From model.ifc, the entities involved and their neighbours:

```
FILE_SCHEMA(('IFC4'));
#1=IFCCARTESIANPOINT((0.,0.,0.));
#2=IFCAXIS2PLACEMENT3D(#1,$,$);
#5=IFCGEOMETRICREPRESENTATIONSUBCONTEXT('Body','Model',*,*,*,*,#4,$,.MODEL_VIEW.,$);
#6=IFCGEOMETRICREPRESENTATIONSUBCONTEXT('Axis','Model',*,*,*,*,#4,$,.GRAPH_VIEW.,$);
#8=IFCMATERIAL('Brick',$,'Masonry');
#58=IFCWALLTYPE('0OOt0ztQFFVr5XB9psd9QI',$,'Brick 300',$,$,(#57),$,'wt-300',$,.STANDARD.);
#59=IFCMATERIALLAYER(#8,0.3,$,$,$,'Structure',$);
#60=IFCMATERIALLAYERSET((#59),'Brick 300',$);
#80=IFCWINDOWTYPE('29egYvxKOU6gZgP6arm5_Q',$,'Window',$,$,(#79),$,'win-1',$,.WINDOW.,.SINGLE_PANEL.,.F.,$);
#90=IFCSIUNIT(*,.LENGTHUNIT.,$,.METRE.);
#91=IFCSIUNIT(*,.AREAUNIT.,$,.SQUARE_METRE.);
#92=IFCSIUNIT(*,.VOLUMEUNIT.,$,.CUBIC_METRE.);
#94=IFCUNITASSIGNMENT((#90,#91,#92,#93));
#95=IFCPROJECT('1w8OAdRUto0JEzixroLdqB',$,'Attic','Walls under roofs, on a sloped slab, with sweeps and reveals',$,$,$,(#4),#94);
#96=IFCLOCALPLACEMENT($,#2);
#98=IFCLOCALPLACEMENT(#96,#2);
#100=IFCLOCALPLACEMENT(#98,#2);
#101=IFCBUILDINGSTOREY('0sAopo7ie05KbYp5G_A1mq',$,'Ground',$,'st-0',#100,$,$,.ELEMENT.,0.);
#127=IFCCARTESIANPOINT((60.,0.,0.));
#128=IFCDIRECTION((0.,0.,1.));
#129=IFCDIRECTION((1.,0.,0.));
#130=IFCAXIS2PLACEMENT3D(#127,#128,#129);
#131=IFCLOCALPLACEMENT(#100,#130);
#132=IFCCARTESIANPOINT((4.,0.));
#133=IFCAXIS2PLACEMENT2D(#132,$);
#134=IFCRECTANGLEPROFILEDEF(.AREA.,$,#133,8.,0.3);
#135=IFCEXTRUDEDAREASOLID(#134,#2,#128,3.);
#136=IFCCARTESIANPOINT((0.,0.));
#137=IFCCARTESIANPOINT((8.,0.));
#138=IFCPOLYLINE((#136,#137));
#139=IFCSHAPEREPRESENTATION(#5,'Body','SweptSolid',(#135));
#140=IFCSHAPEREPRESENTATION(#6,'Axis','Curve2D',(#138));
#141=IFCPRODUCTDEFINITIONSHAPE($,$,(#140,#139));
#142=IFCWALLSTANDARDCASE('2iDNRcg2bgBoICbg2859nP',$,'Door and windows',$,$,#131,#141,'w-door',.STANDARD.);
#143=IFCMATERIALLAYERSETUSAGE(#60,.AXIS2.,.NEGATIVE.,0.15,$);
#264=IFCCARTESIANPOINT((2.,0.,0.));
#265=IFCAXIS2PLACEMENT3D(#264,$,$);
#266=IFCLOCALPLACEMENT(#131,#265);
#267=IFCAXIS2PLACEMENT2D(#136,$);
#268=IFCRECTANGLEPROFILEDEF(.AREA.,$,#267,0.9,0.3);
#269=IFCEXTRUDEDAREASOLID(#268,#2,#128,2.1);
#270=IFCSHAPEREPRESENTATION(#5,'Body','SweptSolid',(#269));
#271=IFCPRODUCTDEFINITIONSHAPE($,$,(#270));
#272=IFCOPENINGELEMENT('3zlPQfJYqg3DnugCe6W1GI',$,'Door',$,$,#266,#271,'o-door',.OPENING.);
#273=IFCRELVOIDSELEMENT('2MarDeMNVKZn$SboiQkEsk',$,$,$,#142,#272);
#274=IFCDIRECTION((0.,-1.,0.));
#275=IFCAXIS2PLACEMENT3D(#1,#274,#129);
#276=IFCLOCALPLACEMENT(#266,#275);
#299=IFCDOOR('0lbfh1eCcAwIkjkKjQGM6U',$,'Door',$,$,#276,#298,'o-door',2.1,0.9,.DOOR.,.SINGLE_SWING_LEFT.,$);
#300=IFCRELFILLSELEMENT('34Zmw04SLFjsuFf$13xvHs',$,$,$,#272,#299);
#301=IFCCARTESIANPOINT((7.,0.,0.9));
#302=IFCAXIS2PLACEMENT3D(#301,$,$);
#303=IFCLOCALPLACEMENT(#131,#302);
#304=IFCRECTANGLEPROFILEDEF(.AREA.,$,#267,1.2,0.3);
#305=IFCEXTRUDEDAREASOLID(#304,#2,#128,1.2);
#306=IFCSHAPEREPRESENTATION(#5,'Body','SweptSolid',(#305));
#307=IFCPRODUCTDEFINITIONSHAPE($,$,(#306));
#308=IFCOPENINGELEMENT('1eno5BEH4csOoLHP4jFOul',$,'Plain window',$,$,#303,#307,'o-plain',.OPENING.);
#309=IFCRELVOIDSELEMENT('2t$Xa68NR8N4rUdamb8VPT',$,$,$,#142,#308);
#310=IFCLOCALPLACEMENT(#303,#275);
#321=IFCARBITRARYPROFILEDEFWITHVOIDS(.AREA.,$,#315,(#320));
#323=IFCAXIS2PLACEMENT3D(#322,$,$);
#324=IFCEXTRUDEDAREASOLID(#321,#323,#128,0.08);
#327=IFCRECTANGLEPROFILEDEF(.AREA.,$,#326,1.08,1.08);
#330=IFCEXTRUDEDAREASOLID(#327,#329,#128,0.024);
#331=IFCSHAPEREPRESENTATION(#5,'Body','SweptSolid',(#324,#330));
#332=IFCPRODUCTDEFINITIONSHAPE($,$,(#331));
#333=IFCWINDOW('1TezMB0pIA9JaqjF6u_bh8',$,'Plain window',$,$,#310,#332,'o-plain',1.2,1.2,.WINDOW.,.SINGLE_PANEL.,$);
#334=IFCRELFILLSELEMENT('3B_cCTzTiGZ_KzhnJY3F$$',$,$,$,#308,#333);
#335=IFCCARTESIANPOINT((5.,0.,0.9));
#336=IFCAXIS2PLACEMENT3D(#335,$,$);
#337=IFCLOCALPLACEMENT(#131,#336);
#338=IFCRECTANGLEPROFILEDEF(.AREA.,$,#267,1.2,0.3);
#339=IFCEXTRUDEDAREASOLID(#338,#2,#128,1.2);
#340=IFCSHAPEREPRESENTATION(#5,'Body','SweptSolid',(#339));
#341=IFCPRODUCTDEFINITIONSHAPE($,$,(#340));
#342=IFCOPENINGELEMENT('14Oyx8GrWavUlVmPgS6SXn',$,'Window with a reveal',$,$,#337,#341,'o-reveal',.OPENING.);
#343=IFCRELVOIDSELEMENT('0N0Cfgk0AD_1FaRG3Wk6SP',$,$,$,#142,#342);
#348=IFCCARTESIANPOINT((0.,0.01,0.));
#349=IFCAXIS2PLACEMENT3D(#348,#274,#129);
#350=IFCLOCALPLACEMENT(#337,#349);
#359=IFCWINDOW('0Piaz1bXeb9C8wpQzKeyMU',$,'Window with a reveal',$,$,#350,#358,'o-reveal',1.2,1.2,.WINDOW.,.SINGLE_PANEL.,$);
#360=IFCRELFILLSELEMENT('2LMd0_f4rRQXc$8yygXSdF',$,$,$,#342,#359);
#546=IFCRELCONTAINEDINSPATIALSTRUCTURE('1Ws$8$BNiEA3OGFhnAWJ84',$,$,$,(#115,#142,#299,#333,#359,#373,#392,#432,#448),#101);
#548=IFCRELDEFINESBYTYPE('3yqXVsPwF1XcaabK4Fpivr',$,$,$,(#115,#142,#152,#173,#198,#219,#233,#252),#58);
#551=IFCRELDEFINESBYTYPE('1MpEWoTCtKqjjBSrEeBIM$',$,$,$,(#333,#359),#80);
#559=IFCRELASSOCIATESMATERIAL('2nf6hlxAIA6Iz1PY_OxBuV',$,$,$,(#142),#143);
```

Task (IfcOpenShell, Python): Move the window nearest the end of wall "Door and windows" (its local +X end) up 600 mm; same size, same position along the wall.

```python
import numpy as np
import ifcopenshell
import ifcopenshell.api.geometry
import ifcopenshell.util.placement
import ifcopenshell.util.unit

model = ifcopenshell.open("model.ifc")
unit_scale = ifcopenshell.util.unit.calculate_unit_scale(model)

window = model.by_guid("1TezMB0pIA9JaqjF6u_bh8")
opening = window.FillsVoids[0].RelatingOpeningElement
dz = 0.6

shift = np.array([0.0, 0.0, dz])
# The window is placed relative to its opening, so it follows when the opening moves.
matrix = ifcopenshell.util.placement.get_local_placement(opening.ObjectPlacement)
matrix[:3, 3] += shift
ifcopenshell.api.geometry.edit_object_placement(
    model, product=opening, matrix=matrix, is_si=False, should_transform_children=True
)

print(f"moved by {dz * unit_scale:+.3f} m")

model.write("model_edited.ifc")
```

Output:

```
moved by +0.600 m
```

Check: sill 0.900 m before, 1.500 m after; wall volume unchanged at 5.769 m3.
